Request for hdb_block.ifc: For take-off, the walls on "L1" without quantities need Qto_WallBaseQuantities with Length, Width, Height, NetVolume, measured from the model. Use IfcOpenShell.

First a look at what the model holds.

```python
import ifcopenshell
import ifcopenshell.util.element
import ifcopenshell.util.unit

model = ifcopenshell.open("hdb_block.ifc")
print(model.schema)
for unit_type in ("LENGTHUNIT", "AREAUNIT", "VOLUMEUNIT"):
    print(unit_type, ifcopenshell.util.unit.calculate_unit_scale(model, unit_type))
storey = next(s for s in model.by_type("IfcBuildingStorey") if s.Name == "L1")
walls = [e for e in ifcopenshell.util.element.get_decomposition(storey) if e.is_a("IfcWall")]
for e in sorted(walls, key=lambda e: e.id()):
    print(e.id(), e.is_a(), e.Name, list(ifcopenshell.util.element.get_psets(e, qtos_only=True)), sep=" | ")
```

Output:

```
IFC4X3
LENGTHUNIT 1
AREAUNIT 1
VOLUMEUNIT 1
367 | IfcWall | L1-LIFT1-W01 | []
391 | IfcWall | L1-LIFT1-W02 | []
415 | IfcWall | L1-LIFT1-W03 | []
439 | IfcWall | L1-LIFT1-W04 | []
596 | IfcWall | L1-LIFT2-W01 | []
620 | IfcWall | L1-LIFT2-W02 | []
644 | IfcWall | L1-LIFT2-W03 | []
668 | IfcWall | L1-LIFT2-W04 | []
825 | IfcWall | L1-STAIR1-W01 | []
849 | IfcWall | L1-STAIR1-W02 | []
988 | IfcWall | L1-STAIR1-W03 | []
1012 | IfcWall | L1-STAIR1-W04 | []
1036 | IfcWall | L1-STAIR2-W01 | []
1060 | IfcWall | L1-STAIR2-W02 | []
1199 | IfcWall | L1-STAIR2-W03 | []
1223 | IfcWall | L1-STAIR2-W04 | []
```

```python
import ifcopenshell
import ifcopenshell.api.pset
import ifcopenshell.geom
import ifcopenshell.util.element
import ifcopenshell.util.shape
import ifcopenshell.util.unit

model = ifcopenshell.open("hdb_block.ifc")
unit_scale = ifcopenshell.util.unit.calculate_unit_scale(model)
volume_scale = ifcopenshell.util.unit.calculate_unit_scale(model, "VOLUMEUNIT")
settings = ifcopenshell.geom.settings()

storey = next(s for s in model.by_type("IfcBuildingStorey") if s.Name == "L1")
walls = [e for e in ifcopenshell.util.element.get_decomposition(storey) if e.is_a("IfcWall")]

for e in sorted(walls, key=lambda e: e.id()):
    if ifcopenshell.util.element.get_psets(e, qtos_only=True, should_inherit=False):
        continue
    # Geometry comes back in metres, in the element's own axes.
    shape = ifcopenshell.geom.create_shape(settings, e)
    values = {
        "Length": ifcopenshell.util.shape.get_x(shape.geometry) / unit_scale,
        "Width": ifcopenshell.util.shape.get_y(shape.geometry) / unit_scale,
        "Height": ifcopenshell.util.shape.get_z(shape.geometry) / unit_scale,
        "NetVolume": ifcopenshell.util.shape.get_volume(shape.geometry) / volume_scale,
    }
    qto = ifcopenshell.api.pset.add_qto(model, product=e, name="Qto_WallBaseQuantities")
    ifcopenshell.api.pset.edit_qto(model, qto=qto, properties=values)
    print(e.id(), {k: round(v, 3) for k, v in values.items()})

model.write("hdb_block_v2.ifc")
```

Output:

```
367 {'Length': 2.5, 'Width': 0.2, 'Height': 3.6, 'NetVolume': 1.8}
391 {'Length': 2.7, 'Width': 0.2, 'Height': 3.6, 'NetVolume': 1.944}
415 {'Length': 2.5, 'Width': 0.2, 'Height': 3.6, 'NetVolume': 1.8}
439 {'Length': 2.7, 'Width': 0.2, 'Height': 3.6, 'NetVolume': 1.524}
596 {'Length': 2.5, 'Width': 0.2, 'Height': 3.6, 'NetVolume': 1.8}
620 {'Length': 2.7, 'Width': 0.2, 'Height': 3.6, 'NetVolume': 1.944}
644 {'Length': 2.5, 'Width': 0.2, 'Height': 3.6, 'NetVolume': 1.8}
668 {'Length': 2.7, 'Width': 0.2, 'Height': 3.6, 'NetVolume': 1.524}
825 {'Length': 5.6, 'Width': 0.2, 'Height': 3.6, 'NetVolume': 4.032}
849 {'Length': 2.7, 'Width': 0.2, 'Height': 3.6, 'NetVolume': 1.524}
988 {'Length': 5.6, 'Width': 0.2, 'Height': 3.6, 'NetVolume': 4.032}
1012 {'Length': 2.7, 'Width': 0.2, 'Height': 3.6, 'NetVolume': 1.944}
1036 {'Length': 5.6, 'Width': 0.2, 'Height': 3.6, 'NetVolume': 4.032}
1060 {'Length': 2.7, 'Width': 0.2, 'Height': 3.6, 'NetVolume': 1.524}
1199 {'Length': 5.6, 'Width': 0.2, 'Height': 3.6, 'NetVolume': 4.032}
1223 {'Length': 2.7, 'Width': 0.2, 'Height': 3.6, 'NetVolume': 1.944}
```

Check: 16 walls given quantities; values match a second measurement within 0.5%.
